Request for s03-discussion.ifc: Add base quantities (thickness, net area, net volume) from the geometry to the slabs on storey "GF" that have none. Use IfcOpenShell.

First a look at what the model holds.

```python
import ifcopenshell
import ifcopenshell.util.element
import ifcopenshell.util.unit

model = ifcopenshell.open("s03-discussion.ifc")
print(model.schema)
for unit_type in ("LENGTHUNIT", "AREAUNIT", "VOLUMEUNIT"):
    print(unit_type, ifcopenshell.util.unit.calculate_unit_scale(model, unit_type))
storey = next(s for s in model.by_type("IfcBuildingStorey") if s.Name == "GF")
slabs = [e for e in ifcopenshell.util.element.get_decomposition(storey) if e.is_a("IfcSlab")]
for e in sorted(slabs, key=lambda e: e.id()):
    print(e.id(), e.is_a(), e.Name, list(ifcopenshell.util.element.get_psets(e, qtos_only=True)), sep=" | ")
```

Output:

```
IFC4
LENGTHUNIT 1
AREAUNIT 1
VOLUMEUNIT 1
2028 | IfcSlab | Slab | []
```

```python
import ifcopenshell
import ifcopenshell.api.pset
import ifcopenshell.geom
import ifcopenshell.util.element
import ifcopenshell.util.shape
import ifcopenshell.util.unit

model = ifcopenshell.open("s03-discussion.ifc")
unit_scale = ifcopenshell.util.unit.calculate_unit_scale(model)
area_scale = ifcopenshell.util.unit.calculate_unit_scale(model, "AREAUNIT")
volume_scale = ifcopenshell.util.unit.calculate_unit_scale(model, "VOLUMEUNIT")
settings = ifcopenshell.geom.settings()

storey = next(s for s in model.by_type("IfcBuildingStorey") if s.Name == "GF")
slabs = [e for e in ifcopenshell.util.element.get_decomposition(storey) if e.is_a("IfcSlab")]

for e in sorted(slabs, key=lambda e: e.id()):
    if ifcopenshell.util.element.get_psets(e, qtos_only=True, should_inherit=False):
        continue
    # Geometry comes back in metres, in the element's own axes.
    shape = ifcopenshell.geom.create_shape(settings, e)
    values = {
        "Width": ifcopenshell.util.shape.get_z(shape.geometry) / unit_scale,
        "NetArea": ifcopenshell.util.shape.get_footprint_area(shape.geometry) / area_scale,
        "NetVolume": ifcopenshell.util.shape.get_volume(shape.geometry) / volume_scale,
    }
    qto = ifcopenshell.api.pset.add_qto(model, product=e, name="Qto_SlabBaseQuantities")
    ifcopenshell.api.pset.edit_qto(model, qto=qto, properties=values)
    print(e.id(), {k: round(v, 3) for k, v in values.items()})

model.write("s03-discussion_updated.ifc")
```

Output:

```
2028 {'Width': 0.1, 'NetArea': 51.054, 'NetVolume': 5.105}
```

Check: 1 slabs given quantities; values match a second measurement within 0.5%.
